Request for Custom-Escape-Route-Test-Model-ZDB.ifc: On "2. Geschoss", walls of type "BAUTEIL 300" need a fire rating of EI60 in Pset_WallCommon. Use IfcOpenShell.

First a look at what the model holds.

```python
import ifcopenshell
import ifcopenshell.util.element

model = ifcopenshell.open("Custom-Escape-Route-Test-Model-ZDB.ifc")
print(model.schema)
storey = next(s for s in model.by_type("IfcBuildingStorey") if s.Name == "2. Geschoss")
walls = [e for e in ifcopenshell.util.element.get_decomposition(storey) if e.is_a("IfcWall")]
seen = {}
for e in walls:
    element_type = ifcopenshell.util.element.get_type(e)
    key = (element_type.Name if element_type != e and element_type else None, ifcopenshell.util.element.get_pset(e, "Pset_WallCommon", "FireRating"))
    seen[key] = seen.get(key, 0) + 1
for (name, value), count in sorted(seen.items(), key=str):
    print(count, "x", name, "|", value)
```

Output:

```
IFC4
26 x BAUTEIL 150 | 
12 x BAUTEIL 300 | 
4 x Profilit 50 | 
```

```python
import ifcopenshell
import ifcopenshell.api.pset
import ifcopenshell.util.element

model = ifcopenshell.open("Custom-Escape-Route-Test-Model-ZDB.ifc")

storey = next(s for s in model.by_type("IfcBuildingStorey") if s.Name == "2. Geschoss")
walls = [e for e in ifcopenshell.util.element.get_decomposition(storey) if e.is_a("IfcWall")]

count = 0
for e in walls:
    element_type = ifcopenshell.util.element.get_type(e)
    if element_type in (None, e) or element_type.Name != "BAUTEIL 300":
        continue
    # add_pset returns the element's existing set when there is one.
    pset = ifcopenshell.api.pset.add_pset(model, product=e, name="Pset_WallCommon")
    ifcopenshell.api.pset.edit_pset(model, pset=pset, properties={"FireRating": "EI60"})
    count += 1

print(count, "walls updated")

model.write("Custom-Escape-Route-Test-Model-ZDB-out.ifc")
```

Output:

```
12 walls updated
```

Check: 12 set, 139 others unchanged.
